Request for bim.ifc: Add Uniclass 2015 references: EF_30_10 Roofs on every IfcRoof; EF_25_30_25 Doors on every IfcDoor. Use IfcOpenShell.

First a look at what the model holds.

```python
import ifcopenshell

model = ifcopenshell.open("bim.ifc")
print(model.schema)
print("classifications:", [c.Name for c in model.by_type("IfcClassification")])
for ifc_class in ("IfcDoor", "IfcRoof", "IfcStair", "IfcWall", "IfcWindow"):
    print(ifc_class, len(model.by_type(ifc_class)))
```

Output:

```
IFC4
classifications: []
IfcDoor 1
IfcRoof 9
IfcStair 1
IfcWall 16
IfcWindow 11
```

```python
import ifcopenshell
import ifcopenshell.api.classification

model = ifcopenshell.open("bim.ifc")

system = ifcopenshell.api.classification.add_classification(model, classification="Uniclass 2015")

codes = {
    "IfcRoof": ("EF_30_10", "Roofs"),
    "IfcDoor": ("EF_25_30_25", "Doors"),
}
for ifc_class, (code, name) in codes.items():
    products = model.by_type(ifc_class)
    ifcopenshell.api.classification.add_reference(
        model, products=products, classification=system, identification=code, name=name
    )
    print(code, len(products))

model.write("bim_updated.ifc")
```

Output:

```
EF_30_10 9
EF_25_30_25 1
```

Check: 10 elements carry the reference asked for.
